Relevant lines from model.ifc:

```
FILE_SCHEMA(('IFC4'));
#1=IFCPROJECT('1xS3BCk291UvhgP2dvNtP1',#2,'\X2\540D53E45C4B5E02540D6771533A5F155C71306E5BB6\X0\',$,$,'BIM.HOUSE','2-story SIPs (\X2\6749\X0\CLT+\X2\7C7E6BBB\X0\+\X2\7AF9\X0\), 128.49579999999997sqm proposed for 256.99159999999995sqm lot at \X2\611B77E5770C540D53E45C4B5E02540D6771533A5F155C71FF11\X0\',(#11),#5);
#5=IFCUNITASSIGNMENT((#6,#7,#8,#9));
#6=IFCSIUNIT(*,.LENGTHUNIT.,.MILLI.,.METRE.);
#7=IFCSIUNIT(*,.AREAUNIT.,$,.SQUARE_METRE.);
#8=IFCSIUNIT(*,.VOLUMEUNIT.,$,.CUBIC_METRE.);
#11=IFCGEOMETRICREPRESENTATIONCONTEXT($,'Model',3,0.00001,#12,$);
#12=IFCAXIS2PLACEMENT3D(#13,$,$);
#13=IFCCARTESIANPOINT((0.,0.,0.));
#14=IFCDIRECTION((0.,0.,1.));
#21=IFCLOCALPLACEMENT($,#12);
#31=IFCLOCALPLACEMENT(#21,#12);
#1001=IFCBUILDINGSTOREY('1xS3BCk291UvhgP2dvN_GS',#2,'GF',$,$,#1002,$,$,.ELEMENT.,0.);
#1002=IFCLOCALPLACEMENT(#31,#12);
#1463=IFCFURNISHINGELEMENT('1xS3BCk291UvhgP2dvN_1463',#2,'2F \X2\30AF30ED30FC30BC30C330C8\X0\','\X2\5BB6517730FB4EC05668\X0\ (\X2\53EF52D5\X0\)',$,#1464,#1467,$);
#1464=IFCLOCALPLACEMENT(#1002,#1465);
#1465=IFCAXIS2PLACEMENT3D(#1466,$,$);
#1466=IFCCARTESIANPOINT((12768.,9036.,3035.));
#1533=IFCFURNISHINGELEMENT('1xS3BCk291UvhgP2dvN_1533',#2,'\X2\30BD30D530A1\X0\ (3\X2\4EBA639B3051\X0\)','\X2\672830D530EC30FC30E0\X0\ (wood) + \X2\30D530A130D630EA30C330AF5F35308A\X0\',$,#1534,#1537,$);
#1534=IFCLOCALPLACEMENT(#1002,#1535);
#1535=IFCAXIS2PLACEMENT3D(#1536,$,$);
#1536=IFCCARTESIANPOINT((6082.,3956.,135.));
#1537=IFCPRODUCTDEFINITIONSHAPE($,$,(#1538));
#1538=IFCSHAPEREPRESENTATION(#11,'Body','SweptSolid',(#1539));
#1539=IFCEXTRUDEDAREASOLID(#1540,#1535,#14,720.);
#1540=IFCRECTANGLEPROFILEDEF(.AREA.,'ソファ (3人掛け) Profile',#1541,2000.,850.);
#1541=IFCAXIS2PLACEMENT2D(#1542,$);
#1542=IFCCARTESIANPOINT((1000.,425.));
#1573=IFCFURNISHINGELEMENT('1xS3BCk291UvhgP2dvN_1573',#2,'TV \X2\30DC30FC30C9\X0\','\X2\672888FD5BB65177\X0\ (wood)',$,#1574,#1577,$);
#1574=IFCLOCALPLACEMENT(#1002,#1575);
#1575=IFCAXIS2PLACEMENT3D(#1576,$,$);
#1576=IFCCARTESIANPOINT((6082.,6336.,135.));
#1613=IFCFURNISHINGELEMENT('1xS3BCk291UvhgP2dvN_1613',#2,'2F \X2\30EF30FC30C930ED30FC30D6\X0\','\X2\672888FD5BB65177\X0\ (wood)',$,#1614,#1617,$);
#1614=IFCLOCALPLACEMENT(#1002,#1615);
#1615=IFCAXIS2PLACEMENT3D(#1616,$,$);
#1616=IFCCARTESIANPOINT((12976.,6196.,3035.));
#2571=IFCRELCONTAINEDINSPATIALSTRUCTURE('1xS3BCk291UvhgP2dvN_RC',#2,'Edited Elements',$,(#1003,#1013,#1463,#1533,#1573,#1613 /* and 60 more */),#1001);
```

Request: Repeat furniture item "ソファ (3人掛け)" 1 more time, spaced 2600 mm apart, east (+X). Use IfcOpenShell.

```python
import numpy as np
import ifcopenshell
import ifcopenshell.api.geometry
import ifcopenshell.api.root
import ifcopenshell.util.element
import ifcopenshell.util.placement

model = ifcopenshell.open("model.ifc")


def reuse_history(source, copy):
    """copy_class also copies each property set's owner history, people and application; keep the originals."""
    for rel in copy.IsDefinedBy:
        if rel.is_a("IfcRelDefinesByProperties") and (history := rel.RelatingPropertyDefinition.OwnerHistory):
            rel.RelatingPropertyDefinition.OwnerHistory = source.OwnerHistory
            ifcopenshell.util.element.remove_deep2(model, history)


source = model.by_id(1533)
base = ifcopenshell.util.placement.get_local_placement(source.ObjectPlacement)
step = np.array([1.0, 0.0, 0.0]) * 2600.0

for i in range(1, 2):
    copy = ifcopenshell.api.root.copy_class(model, product=source)
    copy.Representation = ifcopenshell.util.element.copy_deep(
        model, source.Representation, exclude=["IfcGeometricRepresentationContext", "IfcRepresentationMap"]
    )
    reuse_history(source, copy)
    matrix = base.copy()
    matrix[:3, 3] += i * step
    print("added at", matrix[:3, 3].round(3) + 0.0)
    ifcopenshell.api.geometry.edit_object_placement(model, product=copy, matrix=matrix, is_si=False)

model.write("model-out.ifc")
```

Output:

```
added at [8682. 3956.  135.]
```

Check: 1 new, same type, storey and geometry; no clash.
